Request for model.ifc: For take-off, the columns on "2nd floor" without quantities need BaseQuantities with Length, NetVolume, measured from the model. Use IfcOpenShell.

First a look at what the model holds.

```python
import ifcopenshell
import ifcopenshell.util.element
import ifcopenshell.util.unit

model = ifcopenshell.open("model.ifc")
print(model.schema)
for unit_type in ("LENGTHUNIT", "AREAUNIT", "VOLUMEUNIT"):
    print(unit_type, ifcopenshell.util.unit.calculate_unit_scale(model, unit_type))
storey = next(s for s in model.by_type("IfcBuildingStorey") if s.Name == "2nd floor")
columns = [e for e in ifcopenshell.util.element.get_decomposition(storey) if e.is_a("IfcColumn")]
for e in sorted(columns, key=lambda e: e.id()):
    print(e.id(), e.is_a(), e.Name, list(ifcopenshell.util.element.get_psets(e, qtos_only=True)), sep=" | ")
```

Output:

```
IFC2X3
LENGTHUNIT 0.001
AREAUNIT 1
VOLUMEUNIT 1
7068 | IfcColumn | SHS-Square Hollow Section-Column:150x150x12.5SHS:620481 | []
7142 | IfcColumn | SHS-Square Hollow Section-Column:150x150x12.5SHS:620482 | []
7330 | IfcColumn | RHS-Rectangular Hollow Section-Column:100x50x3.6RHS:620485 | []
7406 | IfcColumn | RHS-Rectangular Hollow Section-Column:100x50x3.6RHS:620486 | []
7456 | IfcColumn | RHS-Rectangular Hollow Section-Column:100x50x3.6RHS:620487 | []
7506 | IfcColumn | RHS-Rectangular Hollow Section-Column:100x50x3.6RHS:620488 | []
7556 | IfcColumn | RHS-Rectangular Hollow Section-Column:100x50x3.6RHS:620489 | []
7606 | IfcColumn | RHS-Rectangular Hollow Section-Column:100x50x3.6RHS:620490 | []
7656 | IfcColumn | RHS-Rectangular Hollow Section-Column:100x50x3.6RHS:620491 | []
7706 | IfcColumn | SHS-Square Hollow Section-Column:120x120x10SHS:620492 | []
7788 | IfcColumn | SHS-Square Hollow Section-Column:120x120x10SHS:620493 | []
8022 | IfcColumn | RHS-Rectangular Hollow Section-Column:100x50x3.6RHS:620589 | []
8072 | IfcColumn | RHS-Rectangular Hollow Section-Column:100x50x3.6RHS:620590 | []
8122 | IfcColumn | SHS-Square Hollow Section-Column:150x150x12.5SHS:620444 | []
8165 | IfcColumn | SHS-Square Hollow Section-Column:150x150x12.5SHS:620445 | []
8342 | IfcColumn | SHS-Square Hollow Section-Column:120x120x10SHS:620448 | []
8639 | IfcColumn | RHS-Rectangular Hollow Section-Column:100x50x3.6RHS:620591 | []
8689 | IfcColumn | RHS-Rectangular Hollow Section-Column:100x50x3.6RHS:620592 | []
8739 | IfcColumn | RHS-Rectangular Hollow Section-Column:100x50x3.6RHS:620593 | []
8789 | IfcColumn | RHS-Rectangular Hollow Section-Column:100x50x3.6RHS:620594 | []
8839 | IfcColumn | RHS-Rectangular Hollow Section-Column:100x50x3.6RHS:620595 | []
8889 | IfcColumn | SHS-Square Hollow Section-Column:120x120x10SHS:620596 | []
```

```python
import ifcopenshell
import ifcopenshell.api.pset
import ifcopenshell.geom
import ifcopenshell.util.element
import ifcopenshell.util.shape
import ifcopenshell.util.unit

model = ifcopenshell.open("model.ifc")
unit_scale = ifcopenshell.util.unit.calculate_unit_scale(model)
volume_scale = ifcopenshell.util.unit.calculate_unit_scale(model, "VOLUMEUNIT")
settings = ifcopenshell.geom.settings()

storey = next(s for s in model.by_type("IfcBuildingStorey") if s.Name == "2nd floor")
columns = [e for e in ifcopenshell.util.element.get_decomposition(storey) if e.is_a("IfcColumn")]

for e in sorted(columns, key=lambda e: e.id()):
    if ifcopenshell.util.element.get_psets(e, qtos_only=True, should_inherit=False):
        continue
    # Geometry comes back in metres, in the element's own axes.
    shape = ifcopenshell.geom.create_shape(settings, e)
    values = {
        "Length": ifcopenshell.util.shape.get_z(shape.geometry) / unit_scale,
        "NetVolume": ifcopenshell.util.shape.get_volume(shape.geometry) / volume_scale,
    }
    qto = ifcopenshell.api.pset.add_qto(model, product=e, name="BaseQuantities")
    ifcopenshell.api.pset.edit_qto(model, qto=qto, properties=values)
    print(e.id(), {k: round(v, 3) for k, v in values.items()})

model.write("model_updated.ifc")
```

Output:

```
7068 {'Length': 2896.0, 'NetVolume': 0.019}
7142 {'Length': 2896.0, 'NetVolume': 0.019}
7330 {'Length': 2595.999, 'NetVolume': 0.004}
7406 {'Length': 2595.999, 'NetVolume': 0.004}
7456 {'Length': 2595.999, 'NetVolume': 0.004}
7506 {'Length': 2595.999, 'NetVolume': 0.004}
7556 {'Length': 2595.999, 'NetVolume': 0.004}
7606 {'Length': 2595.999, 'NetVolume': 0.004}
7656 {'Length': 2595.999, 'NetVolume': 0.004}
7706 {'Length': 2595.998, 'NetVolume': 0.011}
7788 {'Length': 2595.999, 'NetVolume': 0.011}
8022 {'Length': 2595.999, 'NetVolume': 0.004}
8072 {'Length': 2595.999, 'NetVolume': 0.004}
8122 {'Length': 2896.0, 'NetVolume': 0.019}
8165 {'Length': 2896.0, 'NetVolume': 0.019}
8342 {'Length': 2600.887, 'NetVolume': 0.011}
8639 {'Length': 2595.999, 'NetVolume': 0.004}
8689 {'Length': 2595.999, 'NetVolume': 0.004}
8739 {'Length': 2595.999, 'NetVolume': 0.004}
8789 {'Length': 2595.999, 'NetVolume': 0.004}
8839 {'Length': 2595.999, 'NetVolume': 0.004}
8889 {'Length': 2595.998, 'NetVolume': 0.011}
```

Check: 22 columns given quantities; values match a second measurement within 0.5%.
